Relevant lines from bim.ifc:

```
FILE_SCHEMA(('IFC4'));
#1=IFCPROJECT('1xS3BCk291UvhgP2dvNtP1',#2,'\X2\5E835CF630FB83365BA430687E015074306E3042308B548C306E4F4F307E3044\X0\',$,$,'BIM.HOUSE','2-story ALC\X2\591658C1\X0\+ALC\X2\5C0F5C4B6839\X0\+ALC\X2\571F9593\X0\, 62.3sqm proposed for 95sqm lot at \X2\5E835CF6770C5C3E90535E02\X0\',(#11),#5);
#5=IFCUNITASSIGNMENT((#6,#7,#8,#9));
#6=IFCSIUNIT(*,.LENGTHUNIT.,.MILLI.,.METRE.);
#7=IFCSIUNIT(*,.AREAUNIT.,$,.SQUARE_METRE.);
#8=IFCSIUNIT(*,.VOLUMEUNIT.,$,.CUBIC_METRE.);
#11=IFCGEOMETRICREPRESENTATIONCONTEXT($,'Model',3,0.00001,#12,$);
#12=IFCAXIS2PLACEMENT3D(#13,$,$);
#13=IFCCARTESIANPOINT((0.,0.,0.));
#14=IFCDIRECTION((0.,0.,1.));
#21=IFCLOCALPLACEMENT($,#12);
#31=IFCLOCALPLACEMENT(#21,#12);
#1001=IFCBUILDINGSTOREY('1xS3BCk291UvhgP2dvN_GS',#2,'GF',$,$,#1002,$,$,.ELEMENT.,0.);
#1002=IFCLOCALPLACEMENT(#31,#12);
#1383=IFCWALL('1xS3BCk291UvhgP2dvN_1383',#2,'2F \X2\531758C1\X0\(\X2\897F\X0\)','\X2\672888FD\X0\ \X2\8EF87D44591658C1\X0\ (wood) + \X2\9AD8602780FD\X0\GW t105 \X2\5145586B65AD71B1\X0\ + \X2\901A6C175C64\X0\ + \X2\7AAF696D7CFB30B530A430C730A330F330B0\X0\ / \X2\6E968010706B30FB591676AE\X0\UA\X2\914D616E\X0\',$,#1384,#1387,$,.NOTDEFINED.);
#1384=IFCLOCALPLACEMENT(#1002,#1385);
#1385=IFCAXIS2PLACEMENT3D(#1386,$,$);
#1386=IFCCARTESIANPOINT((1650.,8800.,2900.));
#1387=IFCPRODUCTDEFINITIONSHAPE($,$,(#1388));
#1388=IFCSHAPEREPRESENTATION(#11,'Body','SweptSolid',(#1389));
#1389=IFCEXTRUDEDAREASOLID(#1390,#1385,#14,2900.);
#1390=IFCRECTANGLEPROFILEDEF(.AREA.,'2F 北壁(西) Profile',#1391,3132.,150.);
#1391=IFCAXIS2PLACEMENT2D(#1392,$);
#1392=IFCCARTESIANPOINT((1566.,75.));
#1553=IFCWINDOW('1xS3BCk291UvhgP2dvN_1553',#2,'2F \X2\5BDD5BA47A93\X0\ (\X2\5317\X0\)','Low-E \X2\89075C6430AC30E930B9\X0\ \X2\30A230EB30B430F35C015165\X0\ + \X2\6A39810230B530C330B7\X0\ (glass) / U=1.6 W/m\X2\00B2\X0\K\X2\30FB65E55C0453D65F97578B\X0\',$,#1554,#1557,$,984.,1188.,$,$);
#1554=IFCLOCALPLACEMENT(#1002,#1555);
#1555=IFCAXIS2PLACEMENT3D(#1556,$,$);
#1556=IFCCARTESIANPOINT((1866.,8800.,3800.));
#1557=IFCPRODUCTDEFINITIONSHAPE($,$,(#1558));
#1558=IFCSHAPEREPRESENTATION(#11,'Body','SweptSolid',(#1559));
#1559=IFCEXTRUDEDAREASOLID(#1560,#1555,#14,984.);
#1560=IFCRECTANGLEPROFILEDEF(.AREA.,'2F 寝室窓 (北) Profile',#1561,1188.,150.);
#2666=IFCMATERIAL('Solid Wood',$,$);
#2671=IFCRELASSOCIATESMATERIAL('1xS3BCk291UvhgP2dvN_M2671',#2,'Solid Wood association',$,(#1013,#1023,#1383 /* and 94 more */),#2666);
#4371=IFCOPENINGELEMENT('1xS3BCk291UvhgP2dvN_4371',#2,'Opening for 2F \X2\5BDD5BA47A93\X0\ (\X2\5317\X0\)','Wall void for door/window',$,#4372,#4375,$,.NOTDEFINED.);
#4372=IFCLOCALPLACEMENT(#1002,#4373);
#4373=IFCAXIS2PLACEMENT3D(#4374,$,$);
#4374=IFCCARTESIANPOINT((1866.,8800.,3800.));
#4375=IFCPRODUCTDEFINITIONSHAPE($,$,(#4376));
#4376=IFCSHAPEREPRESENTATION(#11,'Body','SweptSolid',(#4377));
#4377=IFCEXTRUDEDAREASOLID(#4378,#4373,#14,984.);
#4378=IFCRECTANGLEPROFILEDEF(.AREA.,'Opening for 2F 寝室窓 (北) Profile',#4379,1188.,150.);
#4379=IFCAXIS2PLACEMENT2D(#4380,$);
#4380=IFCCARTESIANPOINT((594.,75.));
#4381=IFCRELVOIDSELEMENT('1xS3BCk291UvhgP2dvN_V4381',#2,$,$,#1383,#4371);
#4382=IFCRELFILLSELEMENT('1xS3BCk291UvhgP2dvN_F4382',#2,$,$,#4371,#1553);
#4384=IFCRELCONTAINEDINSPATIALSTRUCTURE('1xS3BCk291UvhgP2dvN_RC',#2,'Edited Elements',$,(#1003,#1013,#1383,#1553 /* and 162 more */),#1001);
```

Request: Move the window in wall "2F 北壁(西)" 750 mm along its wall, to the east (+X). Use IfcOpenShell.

```python
import ifcopenshell
import ifcopenshell.api.geometry
import ifcopenshell.util.placement

model = ifcopenshell.open("bim.ifc")

window = model.by_id(1553)
opening = window.FillsVoids[0].RelatingOpeningElement
wall = opening.VoidsElements[0].RelatingBuildingElement

wall_matrix = ifcopenshell.util.placement.get_local_placement(wall.ObjectPlacement)
shift = wall_matrix[:3, 0] * 750.0
before = ifcopenshell.util.placement.get_local_placement(window.ObjectPlacement)[:3, 3].copy()

# The window is not placed relative to its opening, so move both.
for product in (opening, window):
    matrix = ifcopenshell.util.placement.get_local_placement(product.ObjectPlacement)
    matrix[:3, 3] += shift
    ifcopenshell.api.geometry.edit_object_placement(model, product=product, matrix=matrix, is_si=False)

after = ifcopenshell.util.placement.get_local_placement(window.ObjectPlacement)[:3, 3]
print("window moved by", (after - before).round(3) + 0.0)

model.write("bim_edited.ifc")
```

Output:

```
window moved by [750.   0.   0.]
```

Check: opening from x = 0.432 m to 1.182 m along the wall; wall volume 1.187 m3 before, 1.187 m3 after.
